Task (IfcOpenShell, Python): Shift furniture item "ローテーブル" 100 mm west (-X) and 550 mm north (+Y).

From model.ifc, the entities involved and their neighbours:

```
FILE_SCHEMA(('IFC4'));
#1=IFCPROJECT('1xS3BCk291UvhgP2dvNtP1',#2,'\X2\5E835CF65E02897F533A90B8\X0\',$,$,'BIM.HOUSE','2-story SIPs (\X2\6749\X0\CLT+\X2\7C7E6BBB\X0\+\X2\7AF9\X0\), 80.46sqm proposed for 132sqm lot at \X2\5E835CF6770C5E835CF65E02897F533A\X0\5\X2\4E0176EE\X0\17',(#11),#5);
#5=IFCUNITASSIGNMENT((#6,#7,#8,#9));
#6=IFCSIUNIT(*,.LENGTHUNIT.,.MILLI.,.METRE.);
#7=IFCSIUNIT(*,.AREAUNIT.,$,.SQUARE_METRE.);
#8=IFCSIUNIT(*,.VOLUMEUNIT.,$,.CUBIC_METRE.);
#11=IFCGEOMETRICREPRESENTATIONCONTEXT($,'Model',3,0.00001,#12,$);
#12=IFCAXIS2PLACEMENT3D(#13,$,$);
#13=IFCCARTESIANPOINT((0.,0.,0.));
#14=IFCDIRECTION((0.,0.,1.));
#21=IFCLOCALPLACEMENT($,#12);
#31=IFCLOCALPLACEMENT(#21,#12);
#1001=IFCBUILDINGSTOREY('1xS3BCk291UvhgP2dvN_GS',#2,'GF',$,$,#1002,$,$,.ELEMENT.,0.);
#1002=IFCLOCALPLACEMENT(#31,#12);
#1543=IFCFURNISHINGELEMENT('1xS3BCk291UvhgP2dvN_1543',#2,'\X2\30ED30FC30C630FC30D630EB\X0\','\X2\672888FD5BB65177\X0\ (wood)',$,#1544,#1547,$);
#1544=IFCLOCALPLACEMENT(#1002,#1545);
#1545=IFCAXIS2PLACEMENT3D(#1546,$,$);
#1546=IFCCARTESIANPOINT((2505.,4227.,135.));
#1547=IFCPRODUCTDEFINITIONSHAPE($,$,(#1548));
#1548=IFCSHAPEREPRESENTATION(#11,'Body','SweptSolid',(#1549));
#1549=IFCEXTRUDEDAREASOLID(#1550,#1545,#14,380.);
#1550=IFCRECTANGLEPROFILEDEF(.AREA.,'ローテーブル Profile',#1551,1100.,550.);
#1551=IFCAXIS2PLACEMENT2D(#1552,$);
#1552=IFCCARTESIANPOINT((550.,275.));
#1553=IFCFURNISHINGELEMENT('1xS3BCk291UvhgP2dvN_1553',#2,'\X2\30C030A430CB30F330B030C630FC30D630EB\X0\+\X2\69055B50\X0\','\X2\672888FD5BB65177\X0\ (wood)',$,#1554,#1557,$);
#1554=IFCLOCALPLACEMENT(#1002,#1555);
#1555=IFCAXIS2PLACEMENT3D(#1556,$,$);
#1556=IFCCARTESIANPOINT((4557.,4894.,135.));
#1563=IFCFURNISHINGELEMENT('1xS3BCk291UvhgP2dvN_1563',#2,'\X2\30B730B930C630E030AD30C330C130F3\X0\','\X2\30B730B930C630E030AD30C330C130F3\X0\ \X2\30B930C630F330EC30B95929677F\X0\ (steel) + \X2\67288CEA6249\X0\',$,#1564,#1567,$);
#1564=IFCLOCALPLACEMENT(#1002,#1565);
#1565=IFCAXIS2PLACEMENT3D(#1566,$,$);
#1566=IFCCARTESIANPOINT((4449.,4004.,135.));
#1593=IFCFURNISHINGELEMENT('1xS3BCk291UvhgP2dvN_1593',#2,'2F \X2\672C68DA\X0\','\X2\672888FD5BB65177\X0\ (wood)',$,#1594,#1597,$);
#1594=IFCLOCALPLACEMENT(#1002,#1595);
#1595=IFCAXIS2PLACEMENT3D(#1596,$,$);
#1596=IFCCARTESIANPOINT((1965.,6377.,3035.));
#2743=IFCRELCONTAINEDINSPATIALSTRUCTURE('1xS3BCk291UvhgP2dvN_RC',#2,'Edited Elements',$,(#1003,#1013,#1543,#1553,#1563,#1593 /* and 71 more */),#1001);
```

```python
import ifcopenshell
import ifcopenshell.api.geometry
import ifcopenshell.util.placement
import ifcopenshell.util.unit

model = ifcopenshell.open("model.ifc")
unit_scale = ifcopenshell.util.unit.calculate_unit_scale(model)

item = model.by_guid("1xS3BCk291UvhgP2dvN_1543")
matrix = ifcopenshell.util.placement.get_local_placement(item.ObjectPlacement)
matrix[0, 3] -= 0.1 / unit_scale
matrix[1, 3] += 0.55 / unit_scale
ifcopenshell.api.geometry.edit_object_placement(model, product=item, matrix=matrix, is_si=False)

print(ifcopenshell.util.placement.get_local_placement(item.ObjectPlacement).round(3) + 0.0)

model.write("model_rev.ifc")
```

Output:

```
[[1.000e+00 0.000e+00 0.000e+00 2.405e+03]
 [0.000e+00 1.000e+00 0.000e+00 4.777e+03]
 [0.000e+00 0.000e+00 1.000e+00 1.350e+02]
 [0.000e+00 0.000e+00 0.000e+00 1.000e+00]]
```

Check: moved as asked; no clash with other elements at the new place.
